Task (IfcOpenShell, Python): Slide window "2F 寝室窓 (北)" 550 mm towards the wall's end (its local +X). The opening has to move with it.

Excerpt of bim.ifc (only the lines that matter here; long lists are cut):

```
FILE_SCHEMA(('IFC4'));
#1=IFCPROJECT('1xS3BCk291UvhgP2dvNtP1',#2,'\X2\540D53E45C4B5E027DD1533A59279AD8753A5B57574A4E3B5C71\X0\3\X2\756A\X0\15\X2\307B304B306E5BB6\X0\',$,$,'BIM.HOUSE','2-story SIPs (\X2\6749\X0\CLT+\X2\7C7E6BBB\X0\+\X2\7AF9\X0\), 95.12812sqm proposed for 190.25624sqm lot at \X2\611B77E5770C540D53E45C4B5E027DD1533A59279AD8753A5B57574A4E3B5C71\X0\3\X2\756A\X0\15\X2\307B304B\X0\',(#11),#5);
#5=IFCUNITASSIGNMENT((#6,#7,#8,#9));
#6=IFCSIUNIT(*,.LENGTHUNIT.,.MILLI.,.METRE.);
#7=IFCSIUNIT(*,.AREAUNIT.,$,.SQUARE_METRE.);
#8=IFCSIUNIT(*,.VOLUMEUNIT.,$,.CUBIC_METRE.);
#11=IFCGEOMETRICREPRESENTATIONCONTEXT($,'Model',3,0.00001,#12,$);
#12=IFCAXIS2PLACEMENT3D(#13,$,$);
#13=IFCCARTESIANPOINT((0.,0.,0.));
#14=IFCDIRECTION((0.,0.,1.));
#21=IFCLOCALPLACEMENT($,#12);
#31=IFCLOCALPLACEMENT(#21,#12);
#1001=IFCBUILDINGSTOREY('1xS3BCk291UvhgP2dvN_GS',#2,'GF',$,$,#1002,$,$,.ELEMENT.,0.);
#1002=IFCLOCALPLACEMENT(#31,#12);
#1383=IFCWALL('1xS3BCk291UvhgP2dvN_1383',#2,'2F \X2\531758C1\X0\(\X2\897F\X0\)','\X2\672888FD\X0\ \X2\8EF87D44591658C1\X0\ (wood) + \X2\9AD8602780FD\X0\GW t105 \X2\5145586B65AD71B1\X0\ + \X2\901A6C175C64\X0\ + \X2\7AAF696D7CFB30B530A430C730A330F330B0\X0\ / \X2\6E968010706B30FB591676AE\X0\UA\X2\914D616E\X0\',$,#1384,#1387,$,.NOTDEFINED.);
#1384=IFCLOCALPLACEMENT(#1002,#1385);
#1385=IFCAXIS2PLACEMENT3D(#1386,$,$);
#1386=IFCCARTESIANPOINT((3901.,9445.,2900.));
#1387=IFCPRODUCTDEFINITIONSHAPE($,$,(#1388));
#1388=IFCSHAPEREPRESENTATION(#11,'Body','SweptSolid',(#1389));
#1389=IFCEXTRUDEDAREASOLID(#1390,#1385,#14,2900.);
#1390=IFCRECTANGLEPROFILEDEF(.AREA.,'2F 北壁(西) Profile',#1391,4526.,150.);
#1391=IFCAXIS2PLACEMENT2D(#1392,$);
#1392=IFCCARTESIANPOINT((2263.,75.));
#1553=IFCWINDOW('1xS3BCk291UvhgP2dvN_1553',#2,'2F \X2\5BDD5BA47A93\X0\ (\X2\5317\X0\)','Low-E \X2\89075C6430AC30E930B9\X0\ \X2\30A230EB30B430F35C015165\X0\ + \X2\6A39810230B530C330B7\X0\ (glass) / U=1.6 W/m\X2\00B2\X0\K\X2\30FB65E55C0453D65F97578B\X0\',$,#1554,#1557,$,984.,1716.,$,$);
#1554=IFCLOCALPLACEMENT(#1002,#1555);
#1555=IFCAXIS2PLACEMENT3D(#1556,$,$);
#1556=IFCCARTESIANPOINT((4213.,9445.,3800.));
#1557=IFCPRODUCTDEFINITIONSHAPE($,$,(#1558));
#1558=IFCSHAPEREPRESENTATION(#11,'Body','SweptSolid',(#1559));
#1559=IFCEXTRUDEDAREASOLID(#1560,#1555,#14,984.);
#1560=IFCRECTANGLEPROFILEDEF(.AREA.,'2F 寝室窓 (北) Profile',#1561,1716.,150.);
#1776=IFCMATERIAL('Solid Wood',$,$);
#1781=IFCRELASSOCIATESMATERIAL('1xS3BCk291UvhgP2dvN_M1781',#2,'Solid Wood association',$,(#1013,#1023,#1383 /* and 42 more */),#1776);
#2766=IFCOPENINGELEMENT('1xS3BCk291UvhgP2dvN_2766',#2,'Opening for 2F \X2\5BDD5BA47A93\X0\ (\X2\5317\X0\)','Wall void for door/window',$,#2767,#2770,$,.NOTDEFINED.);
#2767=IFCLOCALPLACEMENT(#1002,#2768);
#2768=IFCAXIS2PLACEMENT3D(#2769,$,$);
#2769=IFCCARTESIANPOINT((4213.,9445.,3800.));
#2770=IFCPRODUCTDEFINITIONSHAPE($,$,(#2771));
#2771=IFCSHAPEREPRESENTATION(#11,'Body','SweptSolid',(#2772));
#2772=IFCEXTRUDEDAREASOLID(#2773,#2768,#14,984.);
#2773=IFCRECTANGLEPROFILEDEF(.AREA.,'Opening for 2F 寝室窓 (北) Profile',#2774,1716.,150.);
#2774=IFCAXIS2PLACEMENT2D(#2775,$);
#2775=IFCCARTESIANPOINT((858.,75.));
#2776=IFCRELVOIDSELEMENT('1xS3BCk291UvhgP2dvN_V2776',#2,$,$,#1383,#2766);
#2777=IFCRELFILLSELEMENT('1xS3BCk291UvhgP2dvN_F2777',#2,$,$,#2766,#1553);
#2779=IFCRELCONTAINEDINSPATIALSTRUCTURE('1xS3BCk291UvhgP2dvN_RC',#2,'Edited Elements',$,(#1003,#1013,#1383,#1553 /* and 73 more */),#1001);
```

```python
import ifcopenshell
import ifcopenshell.api.geometry
import ifcopenshell.util.placement
import ifcopenshell.util.unit

model = ifcopenshell.open("bim.ifc")
unit_scale = ifcopenshell.util.unit.calculate_unit_scale(model)

window = model.by_guid("1xS3BCk291UvhgP2dvN_1553")
opening = window.FillsVoids[0].RelatingOpeningElement
wall = opening.VoidsElements[0].RelatingBuildingElement

wall_matrix = ifcopenshell.util.placement.get_local_placement(wall.ObjectPlacement)
shift = wall_matrix[:3, 0] * 0.55 / unit_scale
before = ifcopenshell.util.placement.get_local_placement(window.ObjectPlacement)[:3, 3].copy()

# The window is not placed relative to its opening, so move both.
for product in (opening, window):
    matrix = ifcopenshell.util.placement.get_local_placement(product.ObjectPlacement)
    matrix[:3, 3] += shift
    ifcopenshell.api.geometry.edit_object_placement(model, product=product, matrix=matrix, is_si=False)

after = ifcopenshell.util.placement.get_local_placement(window.ObjectPlacement)[:3, 3]
print("window moved by", (after - before).round(3) + 0.0)

model.write("bim_v2.ifc")
```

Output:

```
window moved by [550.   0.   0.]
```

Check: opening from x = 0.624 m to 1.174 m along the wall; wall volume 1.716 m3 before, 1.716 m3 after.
